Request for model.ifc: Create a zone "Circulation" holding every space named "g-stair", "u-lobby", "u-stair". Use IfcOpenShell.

First a look at what the model holds.

```python
import ifcopenshell

model = ifcopenshell.open("model.ifc")
print(model.schema)
seen = {}
for space in model.by_type("IfcSpace"):
    seen[space.LongName] = seen.get(space.LongName, 0) + 1
for name, count in sorted(seen.items(), key=str):
    print(count, "x", name)
print("zones:", [z.Name for z in model.by_type("IfcZone")][:20])
```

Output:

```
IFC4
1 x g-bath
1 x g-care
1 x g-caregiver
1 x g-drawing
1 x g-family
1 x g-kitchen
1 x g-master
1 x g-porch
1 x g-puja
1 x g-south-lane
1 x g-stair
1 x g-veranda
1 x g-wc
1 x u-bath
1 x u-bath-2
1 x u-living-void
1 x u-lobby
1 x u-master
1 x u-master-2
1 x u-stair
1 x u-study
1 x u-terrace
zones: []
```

```python
import ifcopenshell
import ifcopenshell.api.group
import ifcopenshell.api.root

model = ifcopenshell.open("model.ifc")

names = {"g-stair", "u-lobby", "u-stair"}
spaces = [s for s in model.by_type("IfcSpace") if s.LongName in names]

zone = ifcopenshell.api.root.create_entity(model, ifc_class="IfcZone", name="Circulation")
ifcopenshell.api.group.assign_group(model, products=spaces, group=zone)
print(len(spaces), "spaces in", zone.Name)

model.write("model_updated.ifc")
```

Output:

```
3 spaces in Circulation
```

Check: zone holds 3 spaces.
